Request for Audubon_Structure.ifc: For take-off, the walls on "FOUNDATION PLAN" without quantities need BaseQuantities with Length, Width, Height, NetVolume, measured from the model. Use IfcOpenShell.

First a look at what the model holds.

```python
import ifcopenshell
import ifcopenshell.util.element
import ifcopenshell.util.unit

model = ifcopenshell.open("Audubon_Structure.ifc")
print(model.schema)
for unit_type in ("LENGTHUNIT", "AREAUNIT", "VOLUMEUNIT"):
    print(unit_type, ifcopenshell.util.unit.calculate_unit_scale(model, unit_type))
storey = next(s for s in model.by_type("IfcBuildingStorey") if s.Name == "FOUNDATION PLAN")
walls = [e for e in ifcopenshell.util.element.get_decomposition(storey) if e.is_a("IfcWall")]
for e in sorted(walls, key=lambda e: e.id()):
    print(e.id(), e.is_a(), e.Name, list(ifcopenshell.util.element.get_psets(e, qtos_only=True)), sep=" | ")
```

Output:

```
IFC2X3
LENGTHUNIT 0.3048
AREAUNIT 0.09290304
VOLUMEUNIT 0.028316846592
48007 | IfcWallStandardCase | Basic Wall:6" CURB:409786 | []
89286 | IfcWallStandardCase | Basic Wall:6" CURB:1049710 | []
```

```python
import ifcopenshell
import ifcopenshell.api.pset
import ifcopenshell.geom
import ifcopenshell.util.element
import ifcopenshell.util.shape
import ifcopenshell.util.unit

model = ifcopenshell.open("Audubon_Structure.ifc")
unit_scale = ifcopenshell.util.unit.calculate_unit_scale(model)
volume_scale = ifcopenshell.util.unit.calculate_unit_scale(model, "VOLUMEUNIT")
settings = ifcopenshell.geom.settings()

storey = next(s for s in model.by_type("IfcBuildingStorey") if s.Name == "FOUNDATION PLAN")
walls = [e for e in ifcopenshell.util.element.get_decomposition(storey) if e.is_a("IfcWall")]

for e in sorted(walls, key=lambda e: e.id()):
    if ifcopenshell.util.element.get_psets(e, qtos_only=True, should_inherit=False):
        continue
    # Geometry comes back in metres, in the element's own axes.
    shape = ifcopenshell.geom.create_shape(settings, e)
    values = {
        "Length": ifcopenshell.util.shape.get_x(shape.geometry) / unit_scale,
        "Width": ifcopenshell.util.shape.get_y(shape.geometry) / unit_scale,
        "Height": ifcopenshell.util.shape.get_z(shape.geometry) / unit_scale,
        "NetVolume": ifcopenshell.util.shape.get_volume(shape.geometry) / volume_scale,
    }
    qto = ifcopenshell.api.pset.add_qto(model, product=e, name="BaseQuantities")
    ifcopenshell.api.pset.edit_qto(model, qto=qto, properties=values)
    print(e.id(), {k: round(v, 3) for k, v in values.items()})

model.write("Audubon_Structure_rev.ifc")
```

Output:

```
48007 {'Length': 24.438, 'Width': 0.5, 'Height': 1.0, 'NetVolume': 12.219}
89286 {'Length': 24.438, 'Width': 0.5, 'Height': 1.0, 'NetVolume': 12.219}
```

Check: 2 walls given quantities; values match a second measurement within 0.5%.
